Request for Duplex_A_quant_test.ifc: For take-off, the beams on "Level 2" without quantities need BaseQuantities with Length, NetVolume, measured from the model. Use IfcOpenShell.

First a look at what the model holds.

```python
import ifcopenshell
import ifcopenshell.util.element
import ifcopenshell.util.unit

model = ifcopenshell.open("Duplex_A_quant_test.ifc")
print(model.schema)
for unit_type in ("LENGTHUNIT", "AREAUNIT", "VOLUMEUNIT"):
    print(unit_type, ifcopenshell.util.unit.calculate_unit_scale(model, unit_type))
storey = next(s for s in model.by_type("IfcBuildingStorey") if s.Name == "Level 2")
beams = [e for e in ifcopenshell.util.element.get_decomposition(storey) if e.is_a("IfcBeam")]
for e in sorted(beams, key=lambda e: e.id()):
    print(e.id(), e.is_a(), e.Name, list(ifcopenshell.util.element.get_psets(e, qtos_only=True)), sep=" | ")
```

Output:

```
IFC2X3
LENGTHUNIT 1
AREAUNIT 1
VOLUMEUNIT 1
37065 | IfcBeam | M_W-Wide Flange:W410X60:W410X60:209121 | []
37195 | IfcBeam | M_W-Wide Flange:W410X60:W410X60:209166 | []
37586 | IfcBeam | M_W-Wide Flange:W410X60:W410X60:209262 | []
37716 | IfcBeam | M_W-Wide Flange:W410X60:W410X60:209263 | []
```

```python
import ifcopenshell
import ifcopenshell.api.pset
import ifcopenshell.geom
import ifcopenshell.util.element
import ifcopenshell.util.shape
import ifcopenshell.util.unit

model = ifcopenshell.open("Duplex_A_quant_test.ifc")
unit_scale = ifcopenshell.util.unit.calculate_unit_scale(model)
volume_scale = ifcopenshell.util.unit.calculate_unit_scale(model, "VOLUMEUNIT")
settings = ifcopenshell.geom.settings()

storey = next(s for s in model.by_type("IfcBuildingStorey") if s.Name == "Level 2")
beams = [e for e in ifcopenshell.util.element.get_decomposition(storey) if e.is_a("IfcBeam")]

for e in sorted(beams, key=lambda e: e.id()):
    if ifcopenshell.util.element.get_psets(e, qtos_only=True, should_inherit=False):
        continue
    # Geometry comes back in metres, in the element's own axes.
    shape = ifcopenshell.geom.create_shape(settings, e)
    values = {
        "Length": ifcopenshell.util.shape.get_max_xyz(shape.geometry) / unit_scale,
        "NetVolume": ifcopenshell.util.shape.get_volume(shape.geometry) / volume_scale,
    }
    qto = ifcopenshell.api.pset.add_qto(model, product=e, name="BaseQuantities")
    ifcopenshell.api.pset.edit_qto(model, qto=qto, properties=values)
    print(e.id(), {k: round(v, 3) for k, v in values.items()})

model.write("Duplex_A_quant_test_v2.ifc")
```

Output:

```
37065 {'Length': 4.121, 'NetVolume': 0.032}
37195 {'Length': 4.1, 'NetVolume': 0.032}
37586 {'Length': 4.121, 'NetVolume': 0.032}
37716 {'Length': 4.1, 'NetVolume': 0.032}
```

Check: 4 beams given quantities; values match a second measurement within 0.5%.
